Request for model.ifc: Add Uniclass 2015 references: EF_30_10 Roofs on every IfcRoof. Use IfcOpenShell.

First a look at what the model holds.

```python
import ifcopenshell

model = ifcopenshell.open("model.ifc")
print(model.schema)
print("classifications:", [c.Name for c in model.by_type("IfcClassification")])
for ifc_class in ("IfcDoor", "IfcRoof", "IfcStair", "IfcWall", "IfcWindow"):
    print(ifc_class, len(model.by_type(ifc_class)))
```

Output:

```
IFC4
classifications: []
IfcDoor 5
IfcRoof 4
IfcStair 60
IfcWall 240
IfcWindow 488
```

```python
import ifcopenshell
import ifcopenshell.api.classification

model = ifcopenshell.open("model.ifc")

system = ifcopenshell.api.classification.add_classification(model, classification="Uniclass 2015")

codes = {
    "IfcRoof": ("EF_30_10", "Roofs"),
}
for ifc_class, (code, name) in codes.items():
    products = model.by_type(ifc_class)
    ifcopenshell.api.classification.add_reference(
        model, products=products, classification=system, identification=code, name=name
    )
    print(code, len(products))

model.write("model_updated.ifc")
```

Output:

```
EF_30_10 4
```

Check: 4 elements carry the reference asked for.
